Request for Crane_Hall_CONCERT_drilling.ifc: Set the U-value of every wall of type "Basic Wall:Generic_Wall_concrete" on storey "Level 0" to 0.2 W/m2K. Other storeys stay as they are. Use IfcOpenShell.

First a look at what the model holds.

```python
import ifcopenshell
import ifcopenshell.util.element

model = ifcopenshell.open("Crane_Hall_CONCERT_drilling.ifc")
print(model.schema)
storey = next(s for s in model.by_type("IfcBuildingStorey") if s.Name == "Level 0")
walls = [e for e in ifcopenshell.util.element.get_decomposition(storey) if e.is_a("IfcWall")]
seen = {}
for e in walls:
    element_type = ifcopenshell.util.element.get_type(e)
    key = (element_type.Name if element_type != e and element_type else None, ifcopenshell.util.element.get_pset(e, "Pset_WallCommon", "ThermalTransmittance"))
    seen[key] = seen.get(key, 0) + 1
for (name, value), count in sorted(seen.items(), key=str):
    print(count, "x", name, "|", value)
```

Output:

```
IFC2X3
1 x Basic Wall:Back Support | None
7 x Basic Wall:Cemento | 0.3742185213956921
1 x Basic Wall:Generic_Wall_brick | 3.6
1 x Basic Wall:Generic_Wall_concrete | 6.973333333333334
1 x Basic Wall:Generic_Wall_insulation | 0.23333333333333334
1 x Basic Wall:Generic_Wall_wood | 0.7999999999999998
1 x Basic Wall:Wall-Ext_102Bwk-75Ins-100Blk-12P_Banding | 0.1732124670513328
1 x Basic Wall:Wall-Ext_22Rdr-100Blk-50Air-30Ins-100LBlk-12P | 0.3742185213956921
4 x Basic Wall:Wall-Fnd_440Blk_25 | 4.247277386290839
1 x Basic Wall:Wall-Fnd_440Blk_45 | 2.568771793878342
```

```python
import ifcopenshell
import ifcopenshell.api.pset
import ifcopenshell.util.element

model = ifcopenshell.open("Crane_Hall_CONCERT_drilling.ifc")

storey = next(s for s in model.by_type("IfcBuildingStorey") if s.Name == "Level 0")
walls = [e for e in ifcopenshell.util.element.get_decomposition(storey) if e.is_a("IfcWall")]

count = 0
for e in walls:
    element_type = ifcopenshell.util.element.get_type(e)
    if element_type in (None, e) or element_type.Name != "Basic Wall:Generic_Wall_concrete":
        continue
    # add_pset returns the element's existing set when there is one.
    pset = ifcopenshell.api.pset.add_pset(model, product=e, name="Pset_WallCommon")
    ifcopenshell.api.pset.edit_pset(model, pset=pset, properties={"ThermalTransmittance": 0.2})
    count += 1

print(count, "walls updated")

model.write("Crane_Hall_CONCERT_drilling_updated.ifc")
```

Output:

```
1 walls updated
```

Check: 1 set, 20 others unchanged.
